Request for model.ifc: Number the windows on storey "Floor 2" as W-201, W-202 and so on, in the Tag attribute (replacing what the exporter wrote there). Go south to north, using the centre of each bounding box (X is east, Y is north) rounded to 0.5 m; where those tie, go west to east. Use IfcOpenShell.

First a look at what the model holds.

```python
import ifcopenshell
import ifcopenshell.util.element
import ifcopenshell.util.placement

model = ifcopenshell.open("model.ifc")
print(model.schema)
storey = next(s for s in model.by_type("IfcBuildingStorey") if s.Name == "Floor 2")
windows = [e for e in ifcopenshell.util.element.get_decomposition(storey) if e.is_a("IfcWindow")]
for e in sorted(windows, key=lambda e: e.id()):
    origin = ifcopenshell.util.placement.get_local_placement(e.ObjectPlacement)[:3, 3]
    print(e.id(), e.Tag, e.Name, origin.round(2) + 0.0, sep=" | ")
```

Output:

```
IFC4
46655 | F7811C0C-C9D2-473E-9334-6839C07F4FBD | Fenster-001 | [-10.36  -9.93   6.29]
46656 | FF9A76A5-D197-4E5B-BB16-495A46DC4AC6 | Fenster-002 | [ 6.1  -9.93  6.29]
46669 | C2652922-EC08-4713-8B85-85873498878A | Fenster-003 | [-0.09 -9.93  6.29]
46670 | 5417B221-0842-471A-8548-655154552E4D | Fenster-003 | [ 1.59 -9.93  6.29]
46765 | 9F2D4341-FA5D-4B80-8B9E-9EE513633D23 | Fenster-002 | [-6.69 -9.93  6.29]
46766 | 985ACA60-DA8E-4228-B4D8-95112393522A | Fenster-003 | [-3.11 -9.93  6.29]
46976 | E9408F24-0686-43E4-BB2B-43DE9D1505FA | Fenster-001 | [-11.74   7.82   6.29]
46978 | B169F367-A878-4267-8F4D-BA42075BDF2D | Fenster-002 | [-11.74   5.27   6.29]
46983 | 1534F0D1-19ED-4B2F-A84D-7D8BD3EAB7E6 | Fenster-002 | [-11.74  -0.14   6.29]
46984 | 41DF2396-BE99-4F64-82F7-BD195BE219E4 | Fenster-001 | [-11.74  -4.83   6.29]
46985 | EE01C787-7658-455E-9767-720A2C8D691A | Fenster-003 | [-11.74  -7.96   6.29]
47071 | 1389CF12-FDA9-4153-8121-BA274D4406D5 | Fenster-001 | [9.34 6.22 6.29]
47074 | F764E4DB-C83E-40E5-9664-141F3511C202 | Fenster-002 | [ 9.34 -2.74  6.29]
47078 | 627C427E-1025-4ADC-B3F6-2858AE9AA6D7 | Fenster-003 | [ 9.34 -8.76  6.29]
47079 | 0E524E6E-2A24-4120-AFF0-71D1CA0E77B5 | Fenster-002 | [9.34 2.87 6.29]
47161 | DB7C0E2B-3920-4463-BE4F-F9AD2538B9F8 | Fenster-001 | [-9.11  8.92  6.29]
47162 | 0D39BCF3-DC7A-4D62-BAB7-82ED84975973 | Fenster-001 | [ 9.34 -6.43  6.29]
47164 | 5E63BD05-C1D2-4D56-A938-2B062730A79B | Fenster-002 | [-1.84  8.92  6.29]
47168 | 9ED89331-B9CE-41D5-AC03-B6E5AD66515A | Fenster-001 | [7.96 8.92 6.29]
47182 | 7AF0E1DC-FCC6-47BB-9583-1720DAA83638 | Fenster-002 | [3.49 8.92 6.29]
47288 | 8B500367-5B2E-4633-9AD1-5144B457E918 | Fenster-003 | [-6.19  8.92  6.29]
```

```python
import ifcopenshell
import ifcopenshell.geom
import ifcopenshell.util.element
import ifcopenshell.util.shape

model = ifcopenshell.open("model.ifc")
settings = ifcopenshell.geom.settings()
settings.set("use-world-coords", True)


def centre(element):
    shape = ifcopenshell.geom.create_shape(settings, element)
    return ifcopenshell.util.shape.get_bbox_centroid(shape.geometry)


storey = next(s for s in model.by_type("IfcBuildingStorey") if s.Name == "Floor 2")
windows = [e for e in ifcopenshell.util.element.get_decomposition(storey) if e.is_a("IfcWindow")]

# Insertion points can sit at a corner or the storey origin, so sort by the geometry (in metres).
centres = {e: centre(e) for e in windows}
windows.sort(key=lambda e: (round(centres[e][1] / 0.5), centres[e][0]))

for i, e in enumerate(windows, start=1):
    number = f"W-2{i:02d}"
    e.Tag = number
    print(e.id(), number)

model.write("model_edited.ifc")
```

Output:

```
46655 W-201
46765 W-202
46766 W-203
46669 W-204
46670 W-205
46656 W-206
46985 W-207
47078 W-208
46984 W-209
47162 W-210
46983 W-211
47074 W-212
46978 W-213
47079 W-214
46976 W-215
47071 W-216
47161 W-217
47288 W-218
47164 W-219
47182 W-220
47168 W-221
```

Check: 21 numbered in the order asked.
